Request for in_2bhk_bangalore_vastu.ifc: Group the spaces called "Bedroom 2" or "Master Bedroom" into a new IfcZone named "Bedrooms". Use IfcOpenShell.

First a look at what the model holds.

```python
import ifcopenshell

model = ifcopenshell.open("in_2bhk_bangalore_vastu.ifc")
print(model.schema)
seen = {}
for space in model.by_type("IfcSpace"):
    seen[space.LongName] = seen.get(space.LongName, 0) + 1
for name, count in sorted(seen.items(), key=str):
    print(count, "x", name)
print("zones:", [z.Name for z in model.by_type("IfcZone")][:20])
```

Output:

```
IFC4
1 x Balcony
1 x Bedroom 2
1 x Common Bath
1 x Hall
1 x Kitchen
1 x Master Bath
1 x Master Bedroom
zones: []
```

```python
import ifcopenshell
import ifcopenshell.api.group
import ifcopenshell.api.root

model = ifcopenshell.open("in_2bhk_bangalore_vastu.ifc")

names = {"Bedroom 2", "Master Bedroom"}
spaces = [s for s in model.by_type("IfcSpace") if s.LongName in names]

zone = ifcopenshell.api.root.create_entity(model, ifc_class="IfcZone", name="Bedrooms")
ifcopenshell.api.group.assign_group(model, products=spaces, group=zone)
print(len(spaces), "spaces in", zone.Name)

model.write("in_2bhk_bangalore_vastu_edited.ifc")
```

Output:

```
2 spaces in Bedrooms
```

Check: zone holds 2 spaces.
